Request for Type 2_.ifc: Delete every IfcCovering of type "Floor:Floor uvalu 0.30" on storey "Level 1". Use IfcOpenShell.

First a look at what the model holds.

```python
import ifcopenshell
import ifcopenshell.util.element

model = ifcopenshell.open("Type 2_.ifc")
print(model.schema)
storey = next(s for s in model.by_type("IfcBuildingStorey") if s.Name == "Level 1")
coverings = [e for e in ifcopenshell.util.element.get_decomposition(storey) if e.is_a("IfcCovering")]
seen = {}
for e in coverings:
    element_type = ifcopenshell.util.element.get_type(e)
    name = element_type.Name if element_type not in (None, e) else None
    seen[name] = seen.get(name, 0) + 1
for name, count in sorted(seen.items(), key=str):
    print(count, "x", name)
```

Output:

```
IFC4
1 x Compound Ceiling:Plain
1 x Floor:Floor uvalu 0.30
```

```python
import ifcopenshell
import ifcopenshell.api.root
import ifcopenshell.util.element

model = ifcopenshell.open("Type 2_.ifc")

storey = next(s for s in model.by_type("IfcBuildingStorey") if s.Name == "Level 1")
coverings = [e for e in ifcopenshell.util.element.get_decomposition(storey) if e.is_a("IfcCovering")]
targets = [e for e in coverings if (t := ifcopenshell.util.element.get_type(e)) not in (None, e) and t.Name == "Floor:Floor uvalu 0.30"]

for e in targets:
    ifcopenshell.api.root.remove_product(model, product=e)
print(len(targets), "removed")

model.write("Type 2__updated.ifc")
```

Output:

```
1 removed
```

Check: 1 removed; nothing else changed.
